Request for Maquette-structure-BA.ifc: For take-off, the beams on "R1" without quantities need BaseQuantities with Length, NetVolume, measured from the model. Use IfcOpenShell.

First a look at what the model holds.

```python
import ifcopenshell
import ifcopenshell.util.element
import ifcopenshell.util.unit

model = ifcopenshell.open("Maquette-structure-BA.ifc")
print(model.schema)
for unit_type in ("LENGTHUNIT", "AREAUNIT", "VOLUMEUNIT"):
    print(unit_type, ifcopenshell.util.unit.calculate_unit_scale(model, unit_type))
storey = next(s for s in model.by_type("IfcBuildingStorey") if s.Name == "R1")
beams = [e for e in ifcopenshell.util.element.get_decomposition(storey) if e.is_a("IfcBeam")]
for e in sorted(beams, key=lambda e: e.id()):
    print(e.id(), e.is_a(), e.Name, list(ifcopenshell.util.element.get_psets(e, qtos_only=True)), sep=" | ")
```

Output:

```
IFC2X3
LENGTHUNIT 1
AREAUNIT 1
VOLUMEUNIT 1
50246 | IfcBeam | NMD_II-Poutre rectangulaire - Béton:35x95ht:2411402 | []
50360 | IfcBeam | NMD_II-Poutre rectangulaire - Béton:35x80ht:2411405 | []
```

```python
import ifcopenshell
import ifcopenshell.api.pset
import ifcopenshell.geom
import ifcopenshell.util.element
import ifcopenshell.util.shape
import ifcopenshell.util.unit

model = ifcopenshell.open("Maquette-structure-BA.ifc")
unit_scale = ifcopenshell.util.unit.calculate_unit_scale(model)
volume_scale = ifcopenshell.util.unit.calculate_unit_scale(model, "VOLUMEUNIT")
settings = ifcopenshell.geom.settings()

storey = next(s for s in model.by_type("IfcBuildingStorey") if s.Name == "R1")
beams = [e for e in ifcopenshell.util.element.get_decomposition(storey) if e.is_a("IfcBeam")]

for e in sorted(beams, key=lambda e: e.id()):
    if ifcopenshell.util.element.get_psets(e, qtos_only=True, should_inherit=False):
        continue
    # Geometry comes back in metres, in the element's own axes.
    shape = ifcopenshell.geom.create_shape(settings, e)
    values = {
        "Length": ifcopenshell.util.shape.get_max_xyz(shape.geometry) / unit_scale,
        "NetVolume": ifcopenshell.util.shape.get_volume(shape.geometry) / volume_scale,
    }
    qto = ifcopenshell.api.pset.add_qto(model, product=e, name="BaseQuantities")
    ifcopenshell.api.pset.edit_qto(model, qto=qto, properties=values)
    print(e.id(), {k: round(v, 3) for k, v in values.items()})

model.write("Maquette-structure-BA_v2.ifc")
```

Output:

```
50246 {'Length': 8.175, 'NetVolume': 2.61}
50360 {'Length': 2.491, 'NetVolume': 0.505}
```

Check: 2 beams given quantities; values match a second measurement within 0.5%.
